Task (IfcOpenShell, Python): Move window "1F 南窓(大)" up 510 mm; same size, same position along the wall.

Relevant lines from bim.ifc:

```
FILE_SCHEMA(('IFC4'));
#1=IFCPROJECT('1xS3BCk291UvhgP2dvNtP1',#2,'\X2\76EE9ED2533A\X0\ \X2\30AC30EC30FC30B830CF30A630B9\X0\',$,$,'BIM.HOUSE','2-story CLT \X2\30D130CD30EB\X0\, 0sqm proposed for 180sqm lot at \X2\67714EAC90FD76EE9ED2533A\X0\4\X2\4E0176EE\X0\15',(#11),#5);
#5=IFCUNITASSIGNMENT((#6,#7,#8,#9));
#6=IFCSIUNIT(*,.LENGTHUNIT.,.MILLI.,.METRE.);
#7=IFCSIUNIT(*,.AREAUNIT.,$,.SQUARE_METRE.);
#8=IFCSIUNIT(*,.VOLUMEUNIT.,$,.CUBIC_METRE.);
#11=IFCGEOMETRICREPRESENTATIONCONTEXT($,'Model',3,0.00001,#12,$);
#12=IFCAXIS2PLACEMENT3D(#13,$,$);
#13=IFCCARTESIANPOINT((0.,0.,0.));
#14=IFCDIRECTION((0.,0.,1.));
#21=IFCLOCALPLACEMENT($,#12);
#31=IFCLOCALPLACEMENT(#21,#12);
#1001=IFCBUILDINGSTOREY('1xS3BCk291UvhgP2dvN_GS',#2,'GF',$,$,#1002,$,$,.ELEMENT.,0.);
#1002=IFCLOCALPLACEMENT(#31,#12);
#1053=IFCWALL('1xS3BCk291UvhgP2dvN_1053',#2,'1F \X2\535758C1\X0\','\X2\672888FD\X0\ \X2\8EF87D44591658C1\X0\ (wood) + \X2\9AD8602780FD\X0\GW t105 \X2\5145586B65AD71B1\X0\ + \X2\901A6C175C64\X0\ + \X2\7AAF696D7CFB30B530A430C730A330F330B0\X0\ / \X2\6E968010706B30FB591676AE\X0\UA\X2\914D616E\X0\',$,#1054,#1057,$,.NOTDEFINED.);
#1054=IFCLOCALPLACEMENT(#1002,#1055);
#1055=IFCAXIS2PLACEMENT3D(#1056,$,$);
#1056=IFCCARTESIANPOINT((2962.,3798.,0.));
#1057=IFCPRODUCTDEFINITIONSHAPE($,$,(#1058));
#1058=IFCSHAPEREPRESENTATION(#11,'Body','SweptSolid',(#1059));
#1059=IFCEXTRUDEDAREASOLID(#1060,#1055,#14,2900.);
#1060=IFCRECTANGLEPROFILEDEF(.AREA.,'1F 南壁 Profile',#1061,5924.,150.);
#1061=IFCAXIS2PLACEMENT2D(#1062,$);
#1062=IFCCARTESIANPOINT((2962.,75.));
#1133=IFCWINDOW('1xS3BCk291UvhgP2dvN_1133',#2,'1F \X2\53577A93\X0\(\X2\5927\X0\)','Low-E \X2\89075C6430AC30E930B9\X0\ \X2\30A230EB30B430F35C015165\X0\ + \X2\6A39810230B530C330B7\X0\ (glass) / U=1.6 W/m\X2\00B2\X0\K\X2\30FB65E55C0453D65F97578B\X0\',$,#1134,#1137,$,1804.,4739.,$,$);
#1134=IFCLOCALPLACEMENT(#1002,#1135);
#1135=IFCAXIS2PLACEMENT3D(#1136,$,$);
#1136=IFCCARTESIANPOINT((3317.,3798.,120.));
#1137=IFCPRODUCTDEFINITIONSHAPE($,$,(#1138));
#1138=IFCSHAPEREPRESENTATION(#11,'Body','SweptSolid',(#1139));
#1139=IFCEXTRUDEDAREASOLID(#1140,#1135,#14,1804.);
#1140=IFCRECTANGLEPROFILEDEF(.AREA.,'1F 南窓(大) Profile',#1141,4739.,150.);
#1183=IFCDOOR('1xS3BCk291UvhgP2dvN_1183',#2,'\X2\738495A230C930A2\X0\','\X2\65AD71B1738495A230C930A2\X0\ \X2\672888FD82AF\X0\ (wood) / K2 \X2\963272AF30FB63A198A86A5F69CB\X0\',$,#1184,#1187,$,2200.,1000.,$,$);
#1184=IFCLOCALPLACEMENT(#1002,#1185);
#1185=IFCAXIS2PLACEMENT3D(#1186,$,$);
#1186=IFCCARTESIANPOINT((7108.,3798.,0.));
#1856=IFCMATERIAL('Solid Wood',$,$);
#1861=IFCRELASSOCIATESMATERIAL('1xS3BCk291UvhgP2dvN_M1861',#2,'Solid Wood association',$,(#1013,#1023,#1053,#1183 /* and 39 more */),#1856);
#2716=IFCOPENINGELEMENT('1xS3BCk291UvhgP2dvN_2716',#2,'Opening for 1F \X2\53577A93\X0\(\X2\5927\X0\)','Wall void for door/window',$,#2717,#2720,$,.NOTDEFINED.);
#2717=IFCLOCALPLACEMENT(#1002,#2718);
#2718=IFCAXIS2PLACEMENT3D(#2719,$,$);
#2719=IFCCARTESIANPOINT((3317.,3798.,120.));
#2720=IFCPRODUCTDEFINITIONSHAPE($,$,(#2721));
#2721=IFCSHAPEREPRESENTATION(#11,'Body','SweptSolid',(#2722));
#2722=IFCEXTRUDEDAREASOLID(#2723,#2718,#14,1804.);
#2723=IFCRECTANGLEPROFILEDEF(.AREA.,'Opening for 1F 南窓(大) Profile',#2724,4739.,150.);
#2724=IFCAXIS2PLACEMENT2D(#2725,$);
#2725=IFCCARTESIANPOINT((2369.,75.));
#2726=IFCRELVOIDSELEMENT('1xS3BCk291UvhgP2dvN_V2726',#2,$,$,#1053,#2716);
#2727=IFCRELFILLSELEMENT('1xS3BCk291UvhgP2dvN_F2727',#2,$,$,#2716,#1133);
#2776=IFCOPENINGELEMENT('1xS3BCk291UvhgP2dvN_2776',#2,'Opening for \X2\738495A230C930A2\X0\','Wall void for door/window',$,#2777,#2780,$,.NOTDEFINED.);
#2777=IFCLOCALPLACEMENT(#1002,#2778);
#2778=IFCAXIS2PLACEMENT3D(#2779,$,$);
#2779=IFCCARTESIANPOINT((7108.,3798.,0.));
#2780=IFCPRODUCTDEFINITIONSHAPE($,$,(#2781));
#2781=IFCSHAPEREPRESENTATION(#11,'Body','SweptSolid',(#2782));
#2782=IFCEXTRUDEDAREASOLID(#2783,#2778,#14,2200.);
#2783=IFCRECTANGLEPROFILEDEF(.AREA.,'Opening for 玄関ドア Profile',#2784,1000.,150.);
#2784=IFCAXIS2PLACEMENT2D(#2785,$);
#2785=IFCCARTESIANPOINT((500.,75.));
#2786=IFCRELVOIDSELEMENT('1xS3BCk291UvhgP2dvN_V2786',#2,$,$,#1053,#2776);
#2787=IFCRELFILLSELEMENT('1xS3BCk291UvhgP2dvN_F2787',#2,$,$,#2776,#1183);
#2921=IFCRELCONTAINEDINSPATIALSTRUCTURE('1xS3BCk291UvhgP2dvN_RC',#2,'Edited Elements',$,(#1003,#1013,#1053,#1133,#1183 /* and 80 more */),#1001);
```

```python
import numpy as np
import ifcopenshell
import ifcopenshell.api.geometry
import ifcopenshell.util.placement
import ifcopenshell.util.unit

model = ifcopenshell.open("bim.ifc")
unit_scale = ifcopenshell.util.unit.calculate_unit_scale(model)

window = model.by_id(1133)
opening = window.FillsVoids[0].RelatingOpeningElement
dz = 510.0

shift = np.array([0.0, 0.0, dz])
# The window is not placed relative to its opening, so move both.
for product in (opening, window):
    matrix = ifcopenshell.util.placement.get_local_placement(product.ObjectPlacement)
    matrix[:3, 3] += shift
    ifcopenshell.api.geometry.edit_object_placement(model, product=product, matrix=matrix, is_si=False)

print(f"moved by {dz * unit_scale:+.3f} m")

model.write("bim_v2.ifc")
```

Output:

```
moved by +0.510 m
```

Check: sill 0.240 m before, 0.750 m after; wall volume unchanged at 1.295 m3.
